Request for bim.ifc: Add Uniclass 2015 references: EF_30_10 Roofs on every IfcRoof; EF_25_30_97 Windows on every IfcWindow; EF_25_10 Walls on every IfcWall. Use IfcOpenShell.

First a look at what the model holds.

```python
import ifcopenshell

model = ifcopenshell.open("bim.ifc")
print(model.schema)
print("classifications:", [c.Name for c in model.by_type("IfcClassification")])
for ifc_class in ("IfcDoor", "IfcRoof", "IfcStair", "IfcWall", "IfcWindow"):
    print(ifc_class, len(model.by_type(ifc_class)))
```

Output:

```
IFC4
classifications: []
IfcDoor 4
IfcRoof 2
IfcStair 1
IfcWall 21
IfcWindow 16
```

```python
import ifcopenshell
import ifcopenshell.api.classification

model = ifcopenshell.open("bim.ifc")

system = ifcopenshell.api.classification.add_classification(model, classification="Uniclass 2015")

codes = {
    "IfcRoof": ("EF_30_10", "Roofs"),
    "IfcWindow": ("EF_25_30_97", "Windows"),
    "IfcWall": ("EF_25_10", "Walls"),
}
for ifc_class, (code, name) in codes.items():
    products = model.by_type(ifc_class)
    ifcopenshell.api.classification.add_reference(
        model, products=products, classification=system, identification=code, name=name
    )
    print(code, len(products))

model.write("bim_rev.ifc")
```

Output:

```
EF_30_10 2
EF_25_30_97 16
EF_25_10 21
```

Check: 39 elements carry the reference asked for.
